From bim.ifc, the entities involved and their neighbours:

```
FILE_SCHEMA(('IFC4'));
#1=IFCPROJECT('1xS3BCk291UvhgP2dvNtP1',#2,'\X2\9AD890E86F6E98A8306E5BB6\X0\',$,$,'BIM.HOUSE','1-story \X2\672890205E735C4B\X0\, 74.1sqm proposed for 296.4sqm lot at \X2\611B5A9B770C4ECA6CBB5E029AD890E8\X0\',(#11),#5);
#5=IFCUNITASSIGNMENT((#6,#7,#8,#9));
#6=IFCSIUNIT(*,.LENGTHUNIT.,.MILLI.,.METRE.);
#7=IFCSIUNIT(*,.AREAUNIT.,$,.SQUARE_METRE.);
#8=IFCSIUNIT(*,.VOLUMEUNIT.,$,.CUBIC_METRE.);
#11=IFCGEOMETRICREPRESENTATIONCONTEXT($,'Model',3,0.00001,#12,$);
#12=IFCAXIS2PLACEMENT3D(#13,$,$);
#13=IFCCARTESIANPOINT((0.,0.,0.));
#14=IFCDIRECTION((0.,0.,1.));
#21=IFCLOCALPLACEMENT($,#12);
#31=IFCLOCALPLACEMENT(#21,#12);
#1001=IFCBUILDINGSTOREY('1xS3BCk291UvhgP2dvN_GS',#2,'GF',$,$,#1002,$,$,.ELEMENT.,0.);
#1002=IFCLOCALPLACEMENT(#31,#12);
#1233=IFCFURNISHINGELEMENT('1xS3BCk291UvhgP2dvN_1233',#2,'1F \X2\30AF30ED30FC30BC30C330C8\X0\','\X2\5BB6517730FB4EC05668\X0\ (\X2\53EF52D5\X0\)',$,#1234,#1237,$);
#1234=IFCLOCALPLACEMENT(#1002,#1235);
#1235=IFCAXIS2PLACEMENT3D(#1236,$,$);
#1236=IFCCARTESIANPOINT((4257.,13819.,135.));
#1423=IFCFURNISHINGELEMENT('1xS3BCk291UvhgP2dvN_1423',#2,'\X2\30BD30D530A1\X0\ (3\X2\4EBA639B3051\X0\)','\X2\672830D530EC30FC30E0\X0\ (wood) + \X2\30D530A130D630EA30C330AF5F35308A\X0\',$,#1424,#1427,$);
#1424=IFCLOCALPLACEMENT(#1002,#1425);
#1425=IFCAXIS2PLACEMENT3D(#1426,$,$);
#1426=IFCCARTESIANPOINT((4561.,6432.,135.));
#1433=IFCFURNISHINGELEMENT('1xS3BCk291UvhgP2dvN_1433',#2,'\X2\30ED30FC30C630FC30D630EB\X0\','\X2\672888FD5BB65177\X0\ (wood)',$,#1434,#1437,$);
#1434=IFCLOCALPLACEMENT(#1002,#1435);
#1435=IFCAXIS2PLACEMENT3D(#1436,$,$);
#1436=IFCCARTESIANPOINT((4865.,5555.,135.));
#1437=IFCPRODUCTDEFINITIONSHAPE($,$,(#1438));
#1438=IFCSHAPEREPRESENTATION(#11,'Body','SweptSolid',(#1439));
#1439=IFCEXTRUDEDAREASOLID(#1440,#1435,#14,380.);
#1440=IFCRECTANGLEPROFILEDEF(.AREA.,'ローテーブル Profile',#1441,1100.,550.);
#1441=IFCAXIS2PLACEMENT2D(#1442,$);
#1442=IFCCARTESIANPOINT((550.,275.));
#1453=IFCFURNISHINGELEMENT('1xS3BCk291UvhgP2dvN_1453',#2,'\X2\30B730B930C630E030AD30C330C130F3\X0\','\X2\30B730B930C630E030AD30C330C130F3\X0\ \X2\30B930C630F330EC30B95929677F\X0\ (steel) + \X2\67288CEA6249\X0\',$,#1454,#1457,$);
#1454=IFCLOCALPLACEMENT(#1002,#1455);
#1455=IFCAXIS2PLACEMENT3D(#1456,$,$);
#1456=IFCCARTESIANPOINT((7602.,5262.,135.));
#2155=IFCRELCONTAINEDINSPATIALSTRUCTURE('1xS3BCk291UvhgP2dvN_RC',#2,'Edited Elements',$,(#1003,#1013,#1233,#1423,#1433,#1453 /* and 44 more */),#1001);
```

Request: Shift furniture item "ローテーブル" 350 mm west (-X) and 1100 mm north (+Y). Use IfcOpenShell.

```python
import ifcopenshell
import ifcopenshell.api.geometry
import ifcopenshell.util.placement
import ifcopenshell.util.unit

model = ifcopenshell.open("bim.ifc")
unit_scale = ifcopenshell.util.unit.calculate_unit_scale(model)

item = model.by_guid("1xS3BCk291UvhgP2dvN_1433")
matrix = ifcopenshell.util.placement.get_local_placement(item.ObjectPlacement)
matrix[0, 3] -= 0.35 / unit_scale
matrix[1, 3] += 1.1 / unit_scale
ifcopenshell.api.geometry.edit_object_placement(model, product=item, matrix=matrix, is_si=False)

print(ifcopenshell.util.placement.get_local_placement(item.ObjectPlacement).round(3) + 0.0)

model.write("bim-out.ifc")
```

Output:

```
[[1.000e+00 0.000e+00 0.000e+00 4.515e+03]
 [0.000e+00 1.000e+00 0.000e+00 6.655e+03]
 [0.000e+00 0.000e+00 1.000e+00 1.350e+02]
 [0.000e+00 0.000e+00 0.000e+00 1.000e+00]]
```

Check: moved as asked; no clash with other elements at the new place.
